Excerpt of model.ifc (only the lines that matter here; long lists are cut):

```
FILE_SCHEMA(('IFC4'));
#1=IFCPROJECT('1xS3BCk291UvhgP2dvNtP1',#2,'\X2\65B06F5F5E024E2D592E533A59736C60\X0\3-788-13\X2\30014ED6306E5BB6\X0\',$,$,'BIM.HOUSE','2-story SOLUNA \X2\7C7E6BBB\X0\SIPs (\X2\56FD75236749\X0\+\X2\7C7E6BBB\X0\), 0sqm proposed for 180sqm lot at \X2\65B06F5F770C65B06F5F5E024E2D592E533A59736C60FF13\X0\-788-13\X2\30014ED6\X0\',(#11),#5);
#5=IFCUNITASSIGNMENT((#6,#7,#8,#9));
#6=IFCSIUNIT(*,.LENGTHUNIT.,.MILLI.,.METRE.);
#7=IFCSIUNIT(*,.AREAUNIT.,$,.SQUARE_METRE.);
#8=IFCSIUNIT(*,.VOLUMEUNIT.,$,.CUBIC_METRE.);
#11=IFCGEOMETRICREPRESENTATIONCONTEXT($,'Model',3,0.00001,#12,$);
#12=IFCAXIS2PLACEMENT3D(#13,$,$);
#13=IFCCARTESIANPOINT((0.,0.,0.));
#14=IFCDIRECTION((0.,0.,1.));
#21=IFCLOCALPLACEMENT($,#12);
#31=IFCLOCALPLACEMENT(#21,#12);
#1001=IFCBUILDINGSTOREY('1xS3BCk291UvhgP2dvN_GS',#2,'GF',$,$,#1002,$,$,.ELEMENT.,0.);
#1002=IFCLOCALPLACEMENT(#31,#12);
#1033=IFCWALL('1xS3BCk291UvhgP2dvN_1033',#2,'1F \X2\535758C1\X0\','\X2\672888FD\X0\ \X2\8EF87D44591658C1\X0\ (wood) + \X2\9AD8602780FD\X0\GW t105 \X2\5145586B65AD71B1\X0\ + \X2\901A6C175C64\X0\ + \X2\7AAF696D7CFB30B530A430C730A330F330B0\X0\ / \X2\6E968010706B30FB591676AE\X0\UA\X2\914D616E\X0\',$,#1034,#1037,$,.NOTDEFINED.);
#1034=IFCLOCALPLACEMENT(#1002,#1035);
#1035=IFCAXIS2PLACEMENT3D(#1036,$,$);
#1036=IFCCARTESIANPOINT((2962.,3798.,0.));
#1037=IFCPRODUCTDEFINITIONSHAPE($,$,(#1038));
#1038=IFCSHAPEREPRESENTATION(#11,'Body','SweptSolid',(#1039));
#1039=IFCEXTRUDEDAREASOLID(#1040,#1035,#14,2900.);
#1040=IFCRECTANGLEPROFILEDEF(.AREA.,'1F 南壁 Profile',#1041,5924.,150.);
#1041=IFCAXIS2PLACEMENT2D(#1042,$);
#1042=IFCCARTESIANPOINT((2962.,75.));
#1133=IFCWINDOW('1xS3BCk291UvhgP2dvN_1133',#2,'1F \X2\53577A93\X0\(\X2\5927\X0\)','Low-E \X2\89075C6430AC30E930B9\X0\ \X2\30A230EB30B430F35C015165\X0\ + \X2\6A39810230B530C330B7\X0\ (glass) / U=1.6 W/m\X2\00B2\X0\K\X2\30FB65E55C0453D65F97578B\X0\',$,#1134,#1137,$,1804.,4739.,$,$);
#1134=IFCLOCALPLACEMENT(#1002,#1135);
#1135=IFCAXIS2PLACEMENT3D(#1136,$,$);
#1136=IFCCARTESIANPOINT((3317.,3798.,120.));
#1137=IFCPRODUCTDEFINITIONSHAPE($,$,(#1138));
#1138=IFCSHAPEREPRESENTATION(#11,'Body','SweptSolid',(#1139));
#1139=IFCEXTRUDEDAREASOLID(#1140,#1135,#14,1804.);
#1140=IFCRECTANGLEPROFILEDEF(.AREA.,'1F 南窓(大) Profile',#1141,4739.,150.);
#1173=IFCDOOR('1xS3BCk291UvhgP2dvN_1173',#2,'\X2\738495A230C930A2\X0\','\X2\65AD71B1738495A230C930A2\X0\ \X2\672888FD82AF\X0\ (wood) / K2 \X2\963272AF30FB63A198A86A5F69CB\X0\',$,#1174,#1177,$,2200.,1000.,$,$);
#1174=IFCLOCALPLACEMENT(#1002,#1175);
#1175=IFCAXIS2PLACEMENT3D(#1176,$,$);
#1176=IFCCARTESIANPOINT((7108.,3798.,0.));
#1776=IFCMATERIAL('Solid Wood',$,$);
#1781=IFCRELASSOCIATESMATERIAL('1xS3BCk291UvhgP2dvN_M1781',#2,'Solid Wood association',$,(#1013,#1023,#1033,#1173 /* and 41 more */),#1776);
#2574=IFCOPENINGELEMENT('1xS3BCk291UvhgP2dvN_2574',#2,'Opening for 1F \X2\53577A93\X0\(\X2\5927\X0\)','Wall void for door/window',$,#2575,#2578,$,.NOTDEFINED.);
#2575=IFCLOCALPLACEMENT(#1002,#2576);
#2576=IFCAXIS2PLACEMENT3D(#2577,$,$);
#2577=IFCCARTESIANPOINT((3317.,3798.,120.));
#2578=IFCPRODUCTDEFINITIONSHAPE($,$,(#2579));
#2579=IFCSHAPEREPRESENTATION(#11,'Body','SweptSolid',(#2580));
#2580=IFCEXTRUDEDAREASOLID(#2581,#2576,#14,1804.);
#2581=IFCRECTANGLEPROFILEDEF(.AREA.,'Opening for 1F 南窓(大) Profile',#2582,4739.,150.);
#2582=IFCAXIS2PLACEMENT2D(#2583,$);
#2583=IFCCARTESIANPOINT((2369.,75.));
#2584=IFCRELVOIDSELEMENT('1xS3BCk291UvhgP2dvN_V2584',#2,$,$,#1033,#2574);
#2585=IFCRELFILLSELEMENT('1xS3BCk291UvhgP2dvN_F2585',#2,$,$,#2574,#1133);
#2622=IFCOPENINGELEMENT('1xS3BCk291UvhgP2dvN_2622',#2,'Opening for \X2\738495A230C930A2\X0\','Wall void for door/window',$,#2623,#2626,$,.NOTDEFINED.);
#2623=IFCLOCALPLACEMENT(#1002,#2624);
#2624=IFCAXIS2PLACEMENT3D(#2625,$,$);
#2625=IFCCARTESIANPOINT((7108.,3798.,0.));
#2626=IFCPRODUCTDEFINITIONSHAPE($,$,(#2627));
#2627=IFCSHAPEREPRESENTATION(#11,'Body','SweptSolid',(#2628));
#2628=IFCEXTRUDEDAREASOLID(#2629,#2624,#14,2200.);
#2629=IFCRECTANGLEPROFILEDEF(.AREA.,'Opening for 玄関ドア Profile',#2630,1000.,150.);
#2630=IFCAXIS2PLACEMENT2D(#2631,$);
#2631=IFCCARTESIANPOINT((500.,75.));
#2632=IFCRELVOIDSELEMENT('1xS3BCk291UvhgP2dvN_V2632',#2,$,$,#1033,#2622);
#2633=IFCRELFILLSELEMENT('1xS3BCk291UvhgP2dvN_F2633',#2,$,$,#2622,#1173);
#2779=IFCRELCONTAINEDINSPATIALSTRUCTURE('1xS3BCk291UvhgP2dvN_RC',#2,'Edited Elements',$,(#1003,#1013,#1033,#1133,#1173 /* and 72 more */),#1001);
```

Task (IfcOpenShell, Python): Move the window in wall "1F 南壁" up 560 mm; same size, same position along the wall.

```python
import numpy as np
import ifcopenshell
import ifcopenshell.api.geometry
import ifcopenshell.util.placement
import ifcopenshell.util.unit

model = ifcopenshell.open("model.ifc")
unit_scale = ifcopenshell.util.unit.calculate_unit_scale(model)

window = model.by_guid("1xS3BCk291UvhgP2dvN_1133")
opening = window.FillsVoids[0].RelatingOpeningElement
dz = 560.0

shift = np.array([0.0, 0.0, dz])
# The window is not placed relative to its opening, so move both.
for product in (opening, window):
    matrix = ifcopenshell.util.placement.get_local_placement(product.ObjectPlacement)
    matrix[:3, 3] += shift
    ifcopenshell.api.geometry.edit_object_placement(model, product=product, matrix=matrix, is_si=False)

print(f"moved by {dz * unit_scale:+.3f} m")

model.write("model_rev.ifc")
```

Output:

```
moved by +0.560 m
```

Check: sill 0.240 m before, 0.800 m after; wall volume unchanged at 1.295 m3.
